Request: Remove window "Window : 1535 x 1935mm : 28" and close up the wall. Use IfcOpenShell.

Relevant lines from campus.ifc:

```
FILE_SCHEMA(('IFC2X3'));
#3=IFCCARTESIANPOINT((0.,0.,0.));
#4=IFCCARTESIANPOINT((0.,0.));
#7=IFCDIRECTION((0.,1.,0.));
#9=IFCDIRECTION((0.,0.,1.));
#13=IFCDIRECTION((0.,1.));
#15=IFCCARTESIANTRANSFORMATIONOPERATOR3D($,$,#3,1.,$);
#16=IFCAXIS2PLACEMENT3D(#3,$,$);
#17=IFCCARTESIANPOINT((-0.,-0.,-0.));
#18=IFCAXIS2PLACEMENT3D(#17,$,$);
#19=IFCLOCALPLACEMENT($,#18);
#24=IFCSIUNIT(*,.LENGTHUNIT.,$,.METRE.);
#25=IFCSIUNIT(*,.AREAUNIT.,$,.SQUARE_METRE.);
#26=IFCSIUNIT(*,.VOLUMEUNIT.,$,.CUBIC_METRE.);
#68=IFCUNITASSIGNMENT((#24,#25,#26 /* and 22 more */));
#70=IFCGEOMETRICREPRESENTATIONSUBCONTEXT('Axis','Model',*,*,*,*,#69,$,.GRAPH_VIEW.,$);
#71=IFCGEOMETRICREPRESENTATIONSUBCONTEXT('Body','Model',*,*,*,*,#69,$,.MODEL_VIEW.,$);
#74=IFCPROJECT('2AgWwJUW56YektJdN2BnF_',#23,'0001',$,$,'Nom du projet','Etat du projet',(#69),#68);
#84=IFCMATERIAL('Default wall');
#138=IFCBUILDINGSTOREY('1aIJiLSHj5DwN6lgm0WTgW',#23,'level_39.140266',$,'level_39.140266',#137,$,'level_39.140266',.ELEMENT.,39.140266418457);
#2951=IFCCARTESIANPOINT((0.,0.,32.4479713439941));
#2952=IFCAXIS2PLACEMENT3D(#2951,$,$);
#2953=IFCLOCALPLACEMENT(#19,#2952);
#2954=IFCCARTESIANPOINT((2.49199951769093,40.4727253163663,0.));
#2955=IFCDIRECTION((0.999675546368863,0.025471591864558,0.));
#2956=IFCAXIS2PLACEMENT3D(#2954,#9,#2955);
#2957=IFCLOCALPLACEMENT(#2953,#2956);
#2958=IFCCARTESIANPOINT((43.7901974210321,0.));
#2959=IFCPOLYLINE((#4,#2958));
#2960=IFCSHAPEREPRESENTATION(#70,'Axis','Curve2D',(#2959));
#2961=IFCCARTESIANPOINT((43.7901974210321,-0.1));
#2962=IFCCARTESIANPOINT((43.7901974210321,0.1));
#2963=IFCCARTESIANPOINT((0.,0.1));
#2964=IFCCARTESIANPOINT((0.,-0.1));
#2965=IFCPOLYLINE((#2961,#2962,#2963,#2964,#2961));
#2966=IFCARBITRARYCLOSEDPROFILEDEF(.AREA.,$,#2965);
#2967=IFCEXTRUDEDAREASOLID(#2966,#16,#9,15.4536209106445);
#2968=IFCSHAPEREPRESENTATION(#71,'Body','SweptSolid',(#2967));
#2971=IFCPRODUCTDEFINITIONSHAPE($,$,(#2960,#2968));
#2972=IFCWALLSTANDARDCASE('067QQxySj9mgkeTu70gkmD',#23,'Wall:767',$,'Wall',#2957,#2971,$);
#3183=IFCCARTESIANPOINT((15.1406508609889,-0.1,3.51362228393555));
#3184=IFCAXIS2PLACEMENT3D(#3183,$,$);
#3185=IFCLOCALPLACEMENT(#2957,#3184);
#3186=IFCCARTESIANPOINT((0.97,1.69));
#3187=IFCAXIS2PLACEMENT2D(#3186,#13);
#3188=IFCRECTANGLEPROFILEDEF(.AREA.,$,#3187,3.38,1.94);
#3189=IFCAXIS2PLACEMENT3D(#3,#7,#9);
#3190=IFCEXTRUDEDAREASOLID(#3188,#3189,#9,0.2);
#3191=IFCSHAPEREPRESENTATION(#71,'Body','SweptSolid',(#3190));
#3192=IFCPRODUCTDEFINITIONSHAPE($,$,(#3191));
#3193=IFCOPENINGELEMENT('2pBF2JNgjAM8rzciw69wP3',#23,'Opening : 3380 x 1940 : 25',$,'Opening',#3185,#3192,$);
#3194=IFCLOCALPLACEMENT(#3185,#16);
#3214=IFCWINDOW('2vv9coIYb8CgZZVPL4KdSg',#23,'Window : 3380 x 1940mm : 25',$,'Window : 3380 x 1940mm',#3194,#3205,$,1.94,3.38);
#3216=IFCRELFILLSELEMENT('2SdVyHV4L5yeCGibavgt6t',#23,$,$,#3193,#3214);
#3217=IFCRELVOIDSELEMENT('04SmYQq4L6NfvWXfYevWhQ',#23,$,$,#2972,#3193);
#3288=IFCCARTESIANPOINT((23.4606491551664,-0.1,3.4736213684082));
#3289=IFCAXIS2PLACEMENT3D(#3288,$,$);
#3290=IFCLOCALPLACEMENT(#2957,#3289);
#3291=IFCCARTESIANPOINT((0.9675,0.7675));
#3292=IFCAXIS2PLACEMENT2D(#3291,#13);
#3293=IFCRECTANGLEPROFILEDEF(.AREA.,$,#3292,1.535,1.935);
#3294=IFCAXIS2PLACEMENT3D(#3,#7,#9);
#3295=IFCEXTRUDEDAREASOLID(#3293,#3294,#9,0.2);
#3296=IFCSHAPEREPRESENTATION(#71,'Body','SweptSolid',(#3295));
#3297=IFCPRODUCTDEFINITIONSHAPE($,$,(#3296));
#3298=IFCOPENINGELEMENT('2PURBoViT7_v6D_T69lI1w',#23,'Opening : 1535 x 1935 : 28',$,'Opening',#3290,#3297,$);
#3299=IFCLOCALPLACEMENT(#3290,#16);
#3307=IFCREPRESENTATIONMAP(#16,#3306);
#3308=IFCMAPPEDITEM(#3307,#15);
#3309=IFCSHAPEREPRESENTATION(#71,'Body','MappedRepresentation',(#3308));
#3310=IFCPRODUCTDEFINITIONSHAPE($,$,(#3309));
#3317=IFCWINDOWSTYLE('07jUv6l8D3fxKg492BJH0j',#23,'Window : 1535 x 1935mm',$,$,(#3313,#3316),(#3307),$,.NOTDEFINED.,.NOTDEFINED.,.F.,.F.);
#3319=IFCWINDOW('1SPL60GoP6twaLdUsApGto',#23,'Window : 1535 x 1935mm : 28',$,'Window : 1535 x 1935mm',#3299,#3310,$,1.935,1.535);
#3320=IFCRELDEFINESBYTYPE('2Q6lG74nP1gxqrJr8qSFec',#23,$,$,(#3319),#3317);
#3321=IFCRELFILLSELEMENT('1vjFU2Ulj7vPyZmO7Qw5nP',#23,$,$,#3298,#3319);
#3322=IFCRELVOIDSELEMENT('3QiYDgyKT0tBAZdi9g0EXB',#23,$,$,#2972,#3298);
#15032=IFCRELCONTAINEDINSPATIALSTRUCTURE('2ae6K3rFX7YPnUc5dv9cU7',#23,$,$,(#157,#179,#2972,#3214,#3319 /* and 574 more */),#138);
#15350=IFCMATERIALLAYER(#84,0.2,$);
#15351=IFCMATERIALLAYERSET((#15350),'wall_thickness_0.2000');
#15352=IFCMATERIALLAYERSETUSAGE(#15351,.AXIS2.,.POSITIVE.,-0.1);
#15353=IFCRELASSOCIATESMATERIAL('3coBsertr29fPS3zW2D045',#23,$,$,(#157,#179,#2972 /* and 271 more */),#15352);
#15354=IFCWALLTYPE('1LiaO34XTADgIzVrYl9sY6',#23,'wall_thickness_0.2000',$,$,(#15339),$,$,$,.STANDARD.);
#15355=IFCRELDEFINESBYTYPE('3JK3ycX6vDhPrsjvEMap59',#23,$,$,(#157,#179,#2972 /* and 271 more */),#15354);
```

```python
import ifcopenshell
import ifcopenshell.api.feature
import ifcopenshell.api.root
import ifcopenshell.geom
import ifcopenshell.util.shape

model = ifcopenshell.open("campus.ifc")
settings = ifcopenshell.geom.settings()


def volume(element):
    """Net volume in cubic metres, openings subtracted."""
    shape = ifcopenshell.geom.create_shape(settings, element)
    return ifcopenshell.util.shape.get_volume(shape.geometry)


window = model.by_guid("1SPL60GoP6twaLdUsApGto")
opening = window.FillsVoids[0].RelatingOpeningElement
wall = opening.VoidsElements[0].RelatingBuildingElement
before = volume(wall)

ifcopenshell.api.root.remove_product(model, product=window)
ifcopenshell.api.feature.remove_feature(model, feature=opening)

after = volume(wall)

print(f"wall volume {before:.3f} -> {after:.3f} m3")

model.write("campus_updated.ifc")
```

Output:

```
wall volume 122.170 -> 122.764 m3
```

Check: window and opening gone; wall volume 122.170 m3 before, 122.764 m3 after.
